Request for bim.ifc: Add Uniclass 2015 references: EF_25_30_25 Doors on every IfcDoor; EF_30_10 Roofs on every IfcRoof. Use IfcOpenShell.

First a look at what the model holds.

```python
import ifcopenshell

model = ifcopenshell.open("bim.ifc")
print(model.schema)
print("classifications:", [c.Name for c in model.by_type("IfcClassification")])
for ifc_class in ("IfcDoor", "IfcRoof", "IfcStair", "IfcWall", "IfcWindow"):
    print(ifc_class, len(model.by_type(ifc_class)))
```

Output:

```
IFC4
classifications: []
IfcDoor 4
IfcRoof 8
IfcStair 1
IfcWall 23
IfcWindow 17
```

```python
import ifcopenshell
import ifcopenshell.api.classification

model = ifcopenshell.open("bim.ifc")

system = ifcopenshell.api.classification.add_classification(model, classification="Uniclass 2015")

codes = {
    "IfcDoor": ("EF_25_30_25", "Doors"),
    "IfcRoof": ("EF_30_10", "Roofs"),
}
for ifc_class, (code, name) in codes.items():
    products = model.by_type(ifc_class)
    ifcopenshell.api.classification.add_reference(
        model, products=products, classification=system, identification=code, name=name
    )
    print(code, len(products))

model.write("bim_v2.ifc")
```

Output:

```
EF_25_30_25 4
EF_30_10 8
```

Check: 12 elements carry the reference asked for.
